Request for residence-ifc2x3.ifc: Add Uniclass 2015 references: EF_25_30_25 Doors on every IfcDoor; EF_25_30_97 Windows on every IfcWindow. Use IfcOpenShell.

First a look at what the model holds.

```python
import ifcopenshell

model = ifcopenshell.open("residence-ifc2x3.ifc")
print(model.schema)
print("classifications:", [c.Name for c in model.by_type("IfcClassification")])
for ifc_class in ("IfcDoor", "IfcRoof", "IfcStair", "IfcWall", "IfcWindow"):
    print(ifc_class, len(model.by_type(ifc_class)))
```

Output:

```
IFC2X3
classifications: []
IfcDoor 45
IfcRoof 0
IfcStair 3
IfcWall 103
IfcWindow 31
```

```python
import ifcopenshell
import ifcopenshell.api.classification

model = ifcopenshell.open("residence-ifc2x3.ifc")

# IFC2X3 requires Source and Edition and has no link from the project to the system.
system = model.create_entity("IfcClassification", Source="NBS", Edition="2015", Name="Uniclass 2015")

codes = {
    "IfcDoor": ("EF_25_30_25", "Doors"),
    "IfcWindow": ("EF_25_30_97", "Windows"),
}
for ifc_class, (code, name) in codes.items():
    products = model.by_type(ifc_class)
    ifcopenshell.api.classification.add_reference(
        model, products=products, classification=system, identification=code, name=name
    )
    print(code, len(products))

model.write("residence-ifc2x3-out.ifc")
```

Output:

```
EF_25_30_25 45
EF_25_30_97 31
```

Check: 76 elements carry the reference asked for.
